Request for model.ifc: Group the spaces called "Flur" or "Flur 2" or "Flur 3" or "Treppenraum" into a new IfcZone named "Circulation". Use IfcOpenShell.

First a look at what the model holds.

```python
import ifcopenshell

model = ifcopenshell.open("model.ifc")
print(model.schema)
seen = {}
for space in model.by_type("IfcSpace"):
    seen[space.Name] = seen.get(space.Name, 0) + 1
for name, count in sorted(seen.items(), key=str):
    print(count, "x", name)
print("zones:", [z.Name for z in model.by_type("IfcZone")][:20])
```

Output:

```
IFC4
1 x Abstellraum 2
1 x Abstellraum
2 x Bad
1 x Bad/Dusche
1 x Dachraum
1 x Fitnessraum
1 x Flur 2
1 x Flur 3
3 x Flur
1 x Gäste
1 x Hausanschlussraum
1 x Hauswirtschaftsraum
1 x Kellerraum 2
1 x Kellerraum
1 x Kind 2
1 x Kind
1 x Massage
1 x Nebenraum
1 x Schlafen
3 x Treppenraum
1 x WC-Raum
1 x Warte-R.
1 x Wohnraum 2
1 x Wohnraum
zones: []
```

```python
import ifcopenshell
import ifcopenshell.api.group
import ifcopenshell.api.root

model = ifcopenshell.open("model.ifc")

names = {"Flur", "Flur 2", "Flur 3", "Treppenraum"}
spaces = [s for s in model.by_type("IfcSpace") if s.Name in names]

zone = ifcopenshell.api.root.create_entity(model, ifc_class="IfcZone", name="Circulation")
ifcopenshell.api.group.assign_group(model, products=spaces, group=zone)
print(len(spaces), "spaces in", zone.Name)

model.write("model_edited.ifc")
```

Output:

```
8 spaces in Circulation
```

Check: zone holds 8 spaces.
